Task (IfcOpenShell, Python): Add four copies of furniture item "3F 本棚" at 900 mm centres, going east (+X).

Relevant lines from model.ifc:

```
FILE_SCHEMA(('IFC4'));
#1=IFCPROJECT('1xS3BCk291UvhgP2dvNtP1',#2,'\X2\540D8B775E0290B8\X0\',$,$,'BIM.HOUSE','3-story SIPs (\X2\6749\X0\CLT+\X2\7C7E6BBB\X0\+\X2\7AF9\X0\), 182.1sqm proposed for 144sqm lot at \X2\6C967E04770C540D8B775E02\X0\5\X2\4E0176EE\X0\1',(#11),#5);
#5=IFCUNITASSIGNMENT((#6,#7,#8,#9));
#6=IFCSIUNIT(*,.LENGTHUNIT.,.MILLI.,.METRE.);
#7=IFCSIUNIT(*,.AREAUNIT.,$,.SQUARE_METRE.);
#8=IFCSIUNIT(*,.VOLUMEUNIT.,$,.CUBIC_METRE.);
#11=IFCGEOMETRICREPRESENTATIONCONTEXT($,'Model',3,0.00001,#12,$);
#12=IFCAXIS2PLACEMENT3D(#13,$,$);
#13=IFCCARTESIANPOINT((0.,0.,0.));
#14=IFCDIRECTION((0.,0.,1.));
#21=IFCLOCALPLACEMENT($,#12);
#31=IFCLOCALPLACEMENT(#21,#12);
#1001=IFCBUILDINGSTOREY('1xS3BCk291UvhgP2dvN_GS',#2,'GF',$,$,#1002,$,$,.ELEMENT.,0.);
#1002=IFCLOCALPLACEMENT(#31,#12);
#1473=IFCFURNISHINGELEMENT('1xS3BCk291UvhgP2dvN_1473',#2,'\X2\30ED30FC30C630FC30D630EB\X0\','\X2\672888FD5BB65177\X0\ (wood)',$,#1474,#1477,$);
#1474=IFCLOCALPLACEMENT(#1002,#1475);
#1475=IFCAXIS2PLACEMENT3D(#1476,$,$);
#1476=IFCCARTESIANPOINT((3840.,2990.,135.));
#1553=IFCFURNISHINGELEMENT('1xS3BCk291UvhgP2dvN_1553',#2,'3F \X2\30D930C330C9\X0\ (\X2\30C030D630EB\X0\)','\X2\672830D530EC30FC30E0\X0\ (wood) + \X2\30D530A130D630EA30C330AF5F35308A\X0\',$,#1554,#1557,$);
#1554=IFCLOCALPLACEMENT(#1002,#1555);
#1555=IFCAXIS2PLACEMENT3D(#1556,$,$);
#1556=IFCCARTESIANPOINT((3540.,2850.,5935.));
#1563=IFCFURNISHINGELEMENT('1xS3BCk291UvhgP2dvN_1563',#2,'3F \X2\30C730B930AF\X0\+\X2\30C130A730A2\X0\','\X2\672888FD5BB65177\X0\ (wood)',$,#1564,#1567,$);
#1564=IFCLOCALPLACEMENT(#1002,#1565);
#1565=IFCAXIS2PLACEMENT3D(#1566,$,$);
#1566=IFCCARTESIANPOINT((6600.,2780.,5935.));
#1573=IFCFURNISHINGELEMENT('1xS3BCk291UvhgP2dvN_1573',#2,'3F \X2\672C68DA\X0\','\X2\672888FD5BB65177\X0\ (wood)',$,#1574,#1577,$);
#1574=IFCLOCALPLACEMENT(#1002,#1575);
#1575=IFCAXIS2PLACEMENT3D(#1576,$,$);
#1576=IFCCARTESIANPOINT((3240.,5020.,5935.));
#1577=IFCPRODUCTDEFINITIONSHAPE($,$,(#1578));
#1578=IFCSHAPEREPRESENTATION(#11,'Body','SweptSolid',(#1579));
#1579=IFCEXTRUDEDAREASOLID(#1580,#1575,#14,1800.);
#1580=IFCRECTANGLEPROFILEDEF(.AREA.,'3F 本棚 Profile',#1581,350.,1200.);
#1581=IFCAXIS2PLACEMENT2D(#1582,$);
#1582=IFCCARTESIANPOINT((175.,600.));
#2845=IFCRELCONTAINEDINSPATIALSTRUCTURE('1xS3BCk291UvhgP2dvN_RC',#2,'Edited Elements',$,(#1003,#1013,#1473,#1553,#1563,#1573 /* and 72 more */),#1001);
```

```python
import numpy as np
import ifcopenshell
import ifcopenshell.api.geometry
import ifcopenshell.api.root
import ifcopenshell.util.element
import ifcopenshell.util.placement
import ifcopenshell.util.unit

model = ifcopenshell.open("model.ifc")
unit_scale = ifcopenshell.util.unit.calculate_unit_scale(model)


def reuse_history(source, copy):
    """copy_class also copies each property set's owner history, people and application; keep the originals."""
    for rel in copy.IsDefinedBy:
        if rel.is_a("IfcRelDefinesByProperties") and (history := rel.RelatingPropertyDefinition.OwnerHistory):
            rel.RelatingPropertyDefinition.OwnerHistory = source.OwnerHistory
            ifcopenshell.util.element.remove_deep2(model, history)


source = model.by_id(1573)
base = ifcopenshell.util.placement.get_local_placement(source.ObjectPlacement)
step = np.array([1.0, 0.0, 0.0]) * 0.9 / unit_scale

for i in range(1, 5):
    copy = ifcopenshell.api.root.copy_class(model, product=source)
    copy.Representation = ifcopenshell.util.element.copy_deep(
        model, source.Representation, exclude=["IfcGeometricRepresentationContext", "IfcRepresentationMap"]
    )
    reuse_history(source, copy)
    matrix = base.copy()
    matrix[:3, 3] += i * step
    print("added at", matrix[:3, 3].round(3) + 0.0)
    ifcopenshell.api.geometry.edit_object_placement(model, product=copy, matrix=matrix, is_si=False)

model.write("model_v2.ifc")
```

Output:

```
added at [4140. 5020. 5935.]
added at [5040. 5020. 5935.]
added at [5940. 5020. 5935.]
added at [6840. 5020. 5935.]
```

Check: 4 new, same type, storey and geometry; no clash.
